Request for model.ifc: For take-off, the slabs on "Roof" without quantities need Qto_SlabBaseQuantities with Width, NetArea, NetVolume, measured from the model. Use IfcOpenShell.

First a look at what the model holds.

```python
import ifcopenshell
import ifcopenshell.util.element
import ifcopenshell.util.unit

model = ifcopenshell.open("model.ifc")
print(model.schema)
for unit_type in ("LENGTHUNIT", "AREAUNIT", "VOLUMEUNIT"):
    print(unit_type, ifcopenshell.util.unit.calculate_unit_scale(model, unit_type))
storey = next(s for s in model.by_type("IfcBuildingStorey") if s.Name == "Roof")
slabs = [e for e in ifcopenshell.util.element.get_decomposition(storey) if e.is_a("IfcSlab")]
for e in sorted(slabs, key=lambda e: e.id()):
    print(e.id(), e.is_a(), e.Name, list(ifcopenshell.util.element.get_psets(e, qtos_only=True)), sep=" | ")
```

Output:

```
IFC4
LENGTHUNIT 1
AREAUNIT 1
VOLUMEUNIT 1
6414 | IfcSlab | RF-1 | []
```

```python
import ifcopenshell
import ifcopenshell.api.pset
import ifcopenshell.geom
import ifcopenshell.util.element
import ifcopenshell.util.shape
import ifcopenshell.util.unit

model = ifcopenshell.open("model.ifc")
unit_scale = ifcopenshell.util.unit.calculate_unit_scale(model)
area_scale = ifcopenshell.util.unit.calculate_unit_scale(model, "AREAUNIT")
volume_scale = ifcopenshell.util.unit.calculate_unit_scale(model, "VOLUMEUNIT")
settings = ifcopenshell.geom.settings()

storey = next(s for s in model.by_type("IfcBuildingStorey") if s.Name == "Roof")
slabs = [e for e in ifcopenshell.util.element.get_decomposition(storey) if e.is_a("IfcSlab")]

for e in sorted(slabs, key=lambda e: e.id()):
    if ifcopenshell.util.element.get_psets(e, qtos_only=True, should_inherit=False):
        continue
    # Geometry comes back in metres, in the element's own axes.
    shape = ifcopenshell.geom.create_shape(settings, e)
    values = {
        "Width": ifcopenshell.util.shape.get_z(shape.geometry) / unit_scale,
        "NetArea": ifcopenshell.util.shape.get_footprint_area(shape.geometry) / area_scale,
        "NetVolume": ifcopenshell.util.shape.get_volume(shape.geometry) / volume_scale,
    }
    qto = ifcopenshell.api.pset.add_qto(model, product=e, name="Qto_SlabBaseQuantities")
    ifcopenshell.api.pset.edit_qto(model, qto=qto, properties=values)
    print(e.id(), {k: round(v, 3) for k, v in values.items()})

model.write("model_v2.ifc")
```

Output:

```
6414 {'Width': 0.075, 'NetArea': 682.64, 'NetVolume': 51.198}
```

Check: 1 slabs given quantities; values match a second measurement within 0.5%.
